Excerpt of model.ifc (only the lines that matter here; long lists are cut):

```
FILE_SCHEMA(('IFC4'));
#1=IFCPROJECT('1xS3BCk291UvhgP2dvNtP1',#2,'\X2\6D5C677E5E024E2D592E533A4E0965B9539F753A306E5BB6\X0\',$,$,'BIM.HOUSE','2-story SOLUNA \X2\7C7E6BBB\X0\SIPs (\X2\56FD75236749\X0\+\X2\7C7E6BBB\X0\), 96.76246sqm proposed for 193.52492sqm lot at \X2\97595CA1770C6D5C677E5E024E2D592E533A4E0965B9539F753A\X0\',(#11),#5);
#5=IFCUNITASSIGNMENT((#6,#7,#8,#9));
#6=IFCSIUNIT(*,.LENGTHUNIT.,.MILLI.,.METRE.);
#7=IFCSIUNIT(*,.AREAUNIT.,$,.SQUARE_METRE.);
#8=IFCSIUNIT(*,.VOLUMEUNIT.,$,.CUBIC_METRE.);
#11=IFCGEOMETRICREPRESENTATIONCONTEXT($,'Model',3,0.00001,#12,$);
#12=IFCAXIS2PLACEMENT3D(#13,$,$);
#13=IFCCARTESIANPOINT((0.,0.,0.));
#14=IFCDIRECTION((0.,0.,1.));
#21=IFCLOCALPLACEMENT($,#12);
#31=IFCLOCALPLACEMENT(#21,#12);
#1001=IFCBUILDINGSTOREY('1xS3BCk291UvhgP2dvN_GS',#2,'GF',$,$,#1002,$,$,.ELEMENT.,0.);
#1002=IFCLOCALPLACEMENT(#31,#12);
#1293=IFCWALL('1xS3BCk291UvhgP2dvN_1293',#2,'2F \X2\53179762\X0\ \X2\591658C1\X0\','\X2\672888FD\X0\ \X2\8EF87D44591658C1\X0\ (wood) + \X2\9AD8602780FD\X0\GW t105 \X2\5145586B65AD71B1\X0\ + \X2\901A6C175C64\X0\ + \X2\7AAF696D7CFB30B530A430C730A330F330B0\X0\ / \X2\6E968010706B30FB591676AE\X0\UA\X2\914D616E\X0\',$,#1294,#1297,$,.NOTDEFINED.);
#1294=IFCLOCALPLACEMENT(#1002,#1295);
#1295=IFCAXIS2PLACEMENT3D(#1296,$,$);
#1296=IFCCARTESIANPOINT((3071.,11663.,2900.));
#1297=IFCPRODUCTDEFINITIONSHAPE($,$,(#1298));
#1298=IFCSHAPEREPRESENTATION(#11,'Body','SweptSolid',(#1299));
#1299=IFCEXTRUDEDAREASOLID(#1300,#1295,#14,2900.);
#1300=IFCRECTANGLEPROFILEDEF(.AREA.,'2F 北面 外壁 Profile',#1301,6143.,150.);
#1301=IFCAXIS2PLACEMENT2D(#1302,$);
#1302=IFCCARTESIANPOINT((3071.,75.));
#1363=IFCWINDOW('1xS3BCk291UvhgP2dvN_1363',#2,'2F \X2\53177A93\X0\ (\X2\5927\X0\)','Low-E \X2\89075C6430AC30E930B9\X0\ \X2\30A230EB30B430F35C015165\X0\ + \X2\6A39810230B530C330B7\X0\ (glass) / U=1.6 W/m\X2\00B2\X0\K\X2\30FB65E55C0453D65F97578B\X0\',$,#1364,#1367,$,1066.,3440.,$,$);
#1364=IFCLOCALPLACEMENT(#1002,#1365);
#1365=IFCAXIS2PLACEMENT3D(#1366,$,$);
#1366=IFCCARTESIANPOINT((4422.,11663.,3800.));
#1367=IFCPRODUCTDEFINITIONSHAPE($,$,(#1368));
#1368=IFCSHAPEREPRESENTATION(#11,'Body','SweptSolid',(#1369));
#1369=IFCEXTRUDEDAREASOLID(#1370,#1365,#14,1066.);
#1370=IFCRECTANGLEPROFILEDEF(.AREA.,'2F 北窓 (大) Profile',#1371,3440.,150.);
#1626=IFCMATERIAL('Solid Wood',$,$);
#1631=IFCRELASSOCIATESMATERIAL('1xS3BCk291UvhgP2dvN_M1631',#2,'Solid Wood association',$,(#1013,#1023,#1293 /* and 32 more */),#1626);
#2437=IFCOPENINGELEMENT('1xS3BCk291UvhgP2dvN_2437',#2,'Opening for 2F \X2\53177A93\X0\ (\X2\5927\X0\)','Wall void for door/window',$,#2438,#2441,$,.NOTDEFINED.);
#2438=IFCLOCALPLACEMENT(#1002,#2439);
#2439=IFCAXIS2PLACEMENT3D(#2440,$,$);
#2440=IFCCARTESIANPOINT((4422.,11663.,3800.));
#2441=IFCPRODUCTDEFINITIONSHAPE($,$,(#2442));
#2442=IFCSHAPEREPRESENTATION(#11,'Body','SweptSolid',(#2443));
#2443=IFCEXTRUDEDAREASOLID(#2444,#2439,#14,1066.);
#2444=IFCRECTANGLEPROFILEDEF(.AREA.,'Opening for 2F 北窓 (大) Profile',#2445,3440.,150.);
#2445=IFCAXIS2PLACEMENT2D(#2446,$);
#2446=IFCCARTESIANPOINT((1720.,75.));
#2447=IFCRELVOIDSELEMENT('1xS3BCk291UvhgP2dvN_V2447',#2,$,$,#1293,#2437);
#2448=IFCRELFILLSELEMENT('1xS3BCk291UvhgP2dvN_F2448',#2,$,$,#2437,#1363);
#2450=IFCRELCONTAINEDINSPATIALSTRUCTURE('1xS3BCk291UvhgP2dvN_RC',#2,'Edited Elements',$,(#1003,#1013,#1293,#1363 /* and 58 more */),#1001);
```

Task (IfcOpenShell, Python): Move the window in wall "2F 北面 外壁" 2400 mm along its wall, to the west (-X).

```python
import ifcopenshell
import ifcopenshell.api.geometry
import ifcopenshell.util.placement
import ifcopenshell.util.unit

model = ifcopenshell.open("model.ifc")
unit_scale = ifcopenshell.util.unit.calculate_unit_scale(model)

window = model.by_id(1363)
opening = window.FillsVoids[0].RelatingOpeningElement
wall = opening.VoidsElements[0].RelatingBuildingElement

wall_matrix = ifcopenshell.util.placement.get_local_placement(wall.ObjectPlacement)
shift = wall_matrix[:3, 0] * -2.4 / unit_scale
before = ifcopenshell.util.placement.get_local_placement(window.ObjectPlacement)[:3, 3].copy()

# The window is not placed relative to its opening, so move both.
for product in (opening, window):
    matrix = ifcopenshell.util.placement.get_local_placement(product.ObjectPlacement)
    matrix[:3, 3] += shift
    ifcopenshell.api.geometry.edit_object_placement(model, product=product, matrix=matrix, is_si=False)

after = ifcopenshell.util.placement.get_local_placement(window.ObjectPlacement)[:3, 3]
print("window moved by", (after - before).round(3) + 0.0)

model.write("model-out.ifc")
```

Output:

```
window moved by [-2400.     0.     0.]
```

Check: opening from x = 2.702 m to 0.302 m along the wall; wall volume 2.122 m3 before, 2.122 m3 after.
